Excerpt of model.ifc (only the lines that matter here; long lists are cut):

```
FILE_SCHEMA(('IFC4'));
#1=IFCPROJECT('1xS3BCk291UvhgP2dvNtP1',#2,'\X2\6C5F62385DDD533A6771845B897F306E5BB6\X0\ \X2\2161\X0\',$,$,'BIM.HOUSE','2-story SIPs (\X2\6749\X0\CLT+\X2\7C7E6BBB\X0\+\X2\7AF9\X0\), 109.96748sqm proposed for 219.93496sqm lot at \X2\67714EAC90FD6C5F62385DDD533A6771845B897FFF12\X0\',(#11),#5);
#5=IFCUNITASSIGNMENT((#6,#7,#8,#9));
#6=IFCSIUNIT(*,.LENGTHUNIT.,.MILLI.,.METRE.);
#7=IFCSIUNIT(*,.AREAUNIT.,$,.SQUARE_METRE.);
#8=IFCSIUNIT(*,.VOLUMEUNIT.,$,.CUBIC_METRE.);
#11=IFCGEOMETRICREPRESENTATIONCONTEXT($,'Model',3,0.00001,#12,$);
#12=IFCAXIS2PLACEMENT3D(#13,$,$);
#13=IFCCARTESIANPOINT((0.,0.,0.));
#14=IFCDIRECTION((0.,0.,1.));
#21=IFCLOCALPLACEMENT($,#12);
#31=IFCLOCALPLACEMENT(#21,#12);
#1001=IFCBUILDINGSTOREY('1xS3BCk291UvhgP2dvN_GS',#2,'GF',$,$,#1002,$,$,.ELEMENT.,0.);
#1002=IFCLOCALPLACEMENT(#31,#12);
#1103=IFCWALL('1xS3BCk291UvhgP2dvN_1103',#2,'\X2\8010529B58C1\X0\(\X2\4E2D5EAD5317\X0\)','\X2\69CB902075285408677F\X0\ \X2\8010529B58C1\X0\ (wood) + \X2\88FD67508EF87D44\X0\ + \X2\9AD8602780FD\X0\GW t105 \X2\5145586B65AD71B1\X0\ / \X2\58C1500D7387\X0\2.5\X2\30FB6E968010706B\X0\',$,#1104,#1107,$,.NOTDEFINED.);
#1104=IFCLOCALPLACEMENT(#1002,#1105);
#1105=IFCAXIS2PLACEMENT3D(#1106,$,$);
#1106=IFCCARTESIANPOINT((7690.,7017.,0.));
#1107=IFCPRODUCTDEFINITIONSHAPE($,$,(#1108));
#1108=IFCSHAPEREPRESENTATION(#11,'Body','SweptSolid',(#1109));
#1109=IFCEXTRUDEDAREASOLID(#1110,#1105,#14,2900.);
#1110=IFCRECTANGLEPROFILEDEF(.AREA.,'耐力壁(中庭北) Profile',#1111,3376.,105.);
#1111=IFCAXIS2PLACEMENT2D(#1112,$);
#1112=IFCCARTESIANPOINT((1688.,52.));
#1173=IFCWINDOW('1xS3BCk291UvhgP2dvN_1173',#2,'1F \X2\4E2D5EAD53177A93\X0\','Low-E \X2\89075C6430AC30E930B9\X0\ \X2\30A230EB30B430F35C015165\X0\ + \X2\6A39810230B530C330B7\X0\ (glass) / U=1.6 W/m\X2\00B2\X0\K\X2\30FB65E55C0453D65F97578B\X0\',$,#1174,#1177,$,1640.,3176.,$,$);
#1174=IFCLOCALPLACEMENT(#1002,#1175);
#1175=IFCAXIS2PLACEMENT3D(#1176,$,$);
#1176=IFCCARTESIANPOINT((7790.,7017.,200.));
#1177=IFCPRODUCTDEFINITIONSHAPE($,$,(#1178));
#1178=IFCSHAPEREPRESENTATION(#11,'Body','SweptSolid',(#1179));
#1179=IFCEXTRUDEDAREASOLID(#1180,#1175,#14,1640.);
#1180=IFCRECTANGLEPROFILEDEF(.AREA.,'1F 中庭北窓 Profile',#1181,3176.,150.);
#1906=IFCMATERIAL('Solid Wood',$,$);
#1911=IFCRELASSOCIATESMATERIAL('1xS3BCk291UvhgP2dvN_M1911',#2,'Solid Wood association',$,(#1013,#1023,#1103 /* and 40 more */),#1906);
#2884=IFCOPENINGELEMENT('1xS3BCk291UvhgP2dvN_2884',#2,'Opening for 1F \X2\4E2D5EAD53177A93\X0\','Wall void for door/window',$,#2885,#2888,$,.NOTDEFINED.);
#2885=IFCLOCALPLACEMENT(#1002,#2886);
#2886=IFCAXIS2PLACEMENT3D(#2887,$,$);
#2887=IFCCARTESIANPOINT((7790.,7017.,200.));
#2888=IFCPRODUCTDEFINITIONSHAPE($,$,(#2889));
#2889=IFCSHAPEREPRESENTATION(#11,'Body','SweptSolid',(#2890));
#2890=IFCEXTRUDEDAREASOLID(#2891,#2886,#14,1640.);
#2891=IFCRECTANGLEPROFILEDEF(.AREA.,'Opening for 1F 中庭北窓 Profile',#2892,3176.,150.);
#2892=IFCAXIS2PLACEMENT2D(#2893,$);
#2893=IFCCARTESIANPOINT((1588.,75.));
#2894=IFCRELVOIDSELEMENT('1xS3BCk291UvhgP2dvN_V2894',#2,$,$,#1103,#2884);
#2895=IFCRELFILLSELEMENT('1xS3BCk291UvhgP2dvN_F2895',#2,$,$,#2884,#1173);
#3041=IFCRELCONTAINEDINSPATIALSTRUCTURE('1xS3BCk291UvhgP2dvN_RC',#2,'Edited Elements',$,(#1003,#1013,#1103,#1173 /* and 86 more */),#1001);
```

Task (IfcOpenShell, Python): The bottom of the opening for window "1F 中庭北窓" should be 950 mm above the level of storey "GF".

```python
import numpy as np
import ifcopenshell
import ifcopenshell.api.geometry
import ifcopenshell.geom
import ifcopenshell.util.element
import ifcopenshell.util.placement
import ifcopenshell.util.shape
import ifcopenshell.util.unit

model = ifcopenshell.open("model.ifc")
unit_scale = ifcopenshell.util.unit.calculate_unit_scale(model)

window = model.by_guid("1xS3BCk291UvhgP2dvN_1173")
opening = window.FillsVoids[0].RelatingOpeningElement
storey = ifcopenshell.util.element.get_container(window, ifc_class="IfcBuildingStorey")
level = ifcopenshell.util.placement.get_local_placement(storey.ObjectPlacement)[2, 3]

# The opening's origin need not be at the sill, so measure its lowest point.
shape = ifcopenshell.geom.create_shape(ifcopenshell.geom.settings(), opening)
bottom = ifcopenshell.util.shape.get_shape_bottom_elevation(shape, shape.geometry) / unit_scale
dz = level + 0.95 / unit_scale - bottom

shift = np.array([0.0, 0.0, dz])
# The window is not placed relative to its opening, so move both.
for product in (opening, window):
    matrix = ifcopenshell.util.placement.get_local_placement(product.ObjectPlacement)
    matrix[:3, 3] += shift
    ifcopenshell.api.geometry.edit_object_placement(model, product=product, matrix=matrix, is_si=False)

print(f"moved by {dz * unit_scale:+.3f} m")

model.write("model_rev.ifc")
```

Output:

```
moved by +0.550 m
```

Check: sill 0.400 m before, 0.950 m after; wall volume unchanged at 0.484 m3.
